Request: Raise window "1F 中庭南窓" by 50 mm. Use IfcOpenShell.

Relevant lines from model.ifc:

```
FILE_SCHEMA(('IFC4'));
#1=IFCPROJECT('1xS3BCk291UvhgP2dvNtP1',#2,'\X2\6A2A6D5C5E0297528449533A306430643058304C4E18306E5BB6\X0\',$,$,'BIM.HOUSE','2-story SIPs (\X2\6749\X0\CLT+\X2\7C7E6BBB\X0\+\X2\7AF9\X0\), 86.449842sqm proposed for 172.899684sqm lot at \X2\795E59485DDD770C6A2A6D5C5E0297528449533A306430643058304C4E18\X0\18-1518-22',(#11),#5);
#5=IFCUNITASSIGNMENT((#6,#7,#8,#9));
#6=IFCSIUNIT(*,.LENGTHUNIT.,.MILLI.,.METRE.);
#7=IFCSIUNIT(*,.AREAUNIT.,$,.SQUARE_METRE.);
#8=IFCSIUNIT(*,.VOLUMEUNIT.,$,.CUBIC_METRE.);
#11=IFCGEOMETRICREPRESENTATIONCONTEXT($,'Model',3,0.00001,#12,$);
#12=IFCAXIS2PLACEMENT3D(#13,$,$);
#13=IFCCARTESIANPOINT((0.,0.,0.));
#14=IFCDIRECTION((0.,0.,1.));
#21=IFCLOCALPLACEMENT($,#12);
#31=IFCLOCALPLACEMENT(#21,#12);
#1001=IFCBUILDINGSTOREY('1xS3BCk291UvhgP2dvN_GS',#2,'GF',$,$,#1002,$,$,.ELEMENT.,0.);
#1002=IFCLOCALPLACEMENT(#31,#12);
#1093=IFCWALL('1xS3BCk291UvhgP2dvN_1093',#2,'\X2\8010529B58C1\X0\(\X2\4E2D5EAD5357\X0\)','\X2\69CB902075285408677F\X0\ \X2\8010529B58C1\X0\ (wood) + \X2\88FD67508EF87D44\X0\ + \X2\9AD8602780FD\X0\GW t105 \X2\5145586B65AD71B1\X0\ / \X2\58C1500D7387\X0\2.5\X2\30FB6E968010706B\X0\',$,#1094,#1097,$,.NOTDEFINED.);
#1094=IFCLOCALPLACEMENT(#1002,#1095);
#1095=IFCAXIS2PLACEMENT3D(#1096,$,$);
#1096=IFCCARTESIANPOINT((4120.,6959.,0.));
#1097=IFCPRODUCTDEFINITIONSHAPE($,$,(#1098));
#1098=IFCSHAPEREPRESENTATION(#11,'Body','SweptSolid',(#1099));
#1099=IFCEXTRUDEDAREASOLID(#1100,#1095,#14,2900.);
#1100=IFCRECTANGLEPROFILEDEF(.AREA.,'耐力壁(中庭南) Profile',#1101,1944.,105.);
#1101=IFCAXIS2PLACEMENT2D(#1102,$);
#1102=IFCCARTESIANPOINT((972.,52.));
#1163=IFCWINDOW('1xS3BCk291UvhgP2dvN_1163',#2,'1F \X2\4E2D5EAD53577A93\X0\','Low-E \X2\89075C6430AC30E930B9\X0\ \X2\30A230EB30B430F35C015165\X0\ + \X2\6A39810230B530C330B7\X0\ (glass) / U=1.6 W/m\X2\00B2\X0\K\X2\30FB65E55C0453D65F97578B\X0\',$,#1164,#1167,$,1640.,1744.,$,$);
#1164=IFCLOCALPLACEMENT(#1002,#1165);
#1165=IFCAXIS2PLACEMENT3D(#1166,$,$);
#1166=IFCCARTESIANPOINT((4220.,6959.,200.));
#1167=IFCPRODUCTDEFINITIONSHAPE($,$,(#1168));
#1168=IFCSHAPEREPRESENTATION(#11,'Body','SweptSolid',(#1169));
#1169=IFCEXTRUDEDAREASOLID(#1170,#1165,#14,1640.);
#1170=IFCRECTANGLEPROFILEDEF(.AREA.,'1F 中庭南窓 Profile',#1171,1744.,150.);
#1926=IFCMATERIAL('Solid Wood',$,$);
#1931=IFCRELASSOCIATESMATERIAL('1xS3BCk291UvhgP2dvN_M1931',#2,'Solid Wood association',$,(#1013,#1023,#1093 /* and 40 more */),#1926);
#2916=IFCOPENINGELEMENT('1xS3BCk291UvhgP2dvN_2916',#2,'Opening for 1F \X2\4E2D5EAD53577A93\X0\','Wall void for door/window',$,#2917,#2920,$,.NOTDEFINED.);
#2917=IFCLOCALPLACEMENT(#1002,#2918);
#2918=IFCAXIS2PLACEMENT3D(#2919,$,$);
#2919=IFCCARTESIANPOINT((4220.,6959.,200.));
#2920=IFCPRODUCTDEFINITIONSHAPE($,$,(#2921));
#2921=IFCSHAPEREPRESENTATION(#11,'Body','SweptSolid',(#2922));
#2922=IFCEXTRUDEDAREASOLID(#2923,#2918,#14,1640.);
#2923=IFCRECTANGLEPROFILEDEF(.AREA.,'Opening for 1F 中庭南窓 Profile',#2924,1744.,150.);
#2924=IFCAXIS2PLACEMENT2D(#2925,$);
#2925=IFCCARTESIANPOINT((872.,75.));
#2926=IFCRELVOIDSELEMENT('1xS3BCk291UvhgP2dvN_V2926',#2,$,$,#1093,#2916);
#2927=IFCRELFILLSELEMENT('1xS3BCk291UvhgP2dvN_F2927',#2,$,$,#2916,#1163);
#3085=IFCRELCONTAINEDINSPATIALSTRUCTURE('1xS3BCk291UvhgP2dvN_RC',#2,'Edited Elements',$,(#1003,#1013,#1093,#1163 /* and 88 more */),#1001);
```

```python
import numpy as np
import ifcopenshell
import ifcopenshell.api.geometry
import ifcopenshell.util.placement
import ifcopenshell.util.unit

model = ifcopenshell.open("model.ifc")
unit_scale = ifcopenshell.util.unit.calculate_unit_scale(model)

window = model.by_guid("1xS3BCk291UvhgP2dvN_1163")
opening = window.FillsVoids[0].RelatingOpeningElement
dz = 0.05 / unit_scale

shift = np.array([0.0, 0.0, dz])
# The window is not placed relative to its opening, so move both.
for product in (opening, window):
    matrix = ifcopenshell.util.placement.get_local_placement(product.ObjectPlacement)
    matrix[:3, 3] += shift
    ifcopenshell.api.geometry.edit_object_placement(model, product=product, matrix=matrix, is_si=False)

print(f"moved by {dz * unit_scale:+.3f} m")

model.write("model_updated.ifc")
```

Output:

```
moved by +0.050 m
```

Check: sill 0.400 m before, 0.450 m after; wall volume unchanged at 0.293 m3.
